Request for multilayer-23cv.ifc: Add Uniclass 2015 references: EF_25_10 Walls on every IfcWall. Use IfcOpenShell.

First a look at what the model holds.

```python
import ifcopenshell

model = ifcopenshell.open("multilayer-23cv.ifc")
print(model.schema)
print("classifications:", [c.Name for c in model.by_type("IfcClassification")])
for ifc_class in ("IfcDoor", "IfcRoof", "IfcStair", "IfcWall", "IfcWindow"):
    print(ifc_class, len(model.by_type(ifc_class)))
```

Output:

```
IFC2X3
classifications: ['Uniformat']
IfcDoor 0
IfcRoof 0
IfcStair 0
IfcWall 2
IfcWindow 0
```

```python
import ifcopenshell
import ifcopenshell.api.classification

model = ifcopenshell.open("multilayer-23cv.ifc")

# IFC2X3 requires Source and Edition and has no link from the project to the system.
system = model.create_entity("IfcClassification", Source="NBS", Edition="2015", Name="Uniclass 2015")

codes = {
    "IfcWall": ("EF_25_10", "Walls"),
}
for ifc_class, (code, name) in codes.items():
    products = model.by_type(ifc_class)
    ifcopenshell.api.classification.add_reference(
        model, products=products, classification=system, identification=code, name=name
    )
    print(code, len(products))

model.write("multilayer-23cv-out.ifc")
```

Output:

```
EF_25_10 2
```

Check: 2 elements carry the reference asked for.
